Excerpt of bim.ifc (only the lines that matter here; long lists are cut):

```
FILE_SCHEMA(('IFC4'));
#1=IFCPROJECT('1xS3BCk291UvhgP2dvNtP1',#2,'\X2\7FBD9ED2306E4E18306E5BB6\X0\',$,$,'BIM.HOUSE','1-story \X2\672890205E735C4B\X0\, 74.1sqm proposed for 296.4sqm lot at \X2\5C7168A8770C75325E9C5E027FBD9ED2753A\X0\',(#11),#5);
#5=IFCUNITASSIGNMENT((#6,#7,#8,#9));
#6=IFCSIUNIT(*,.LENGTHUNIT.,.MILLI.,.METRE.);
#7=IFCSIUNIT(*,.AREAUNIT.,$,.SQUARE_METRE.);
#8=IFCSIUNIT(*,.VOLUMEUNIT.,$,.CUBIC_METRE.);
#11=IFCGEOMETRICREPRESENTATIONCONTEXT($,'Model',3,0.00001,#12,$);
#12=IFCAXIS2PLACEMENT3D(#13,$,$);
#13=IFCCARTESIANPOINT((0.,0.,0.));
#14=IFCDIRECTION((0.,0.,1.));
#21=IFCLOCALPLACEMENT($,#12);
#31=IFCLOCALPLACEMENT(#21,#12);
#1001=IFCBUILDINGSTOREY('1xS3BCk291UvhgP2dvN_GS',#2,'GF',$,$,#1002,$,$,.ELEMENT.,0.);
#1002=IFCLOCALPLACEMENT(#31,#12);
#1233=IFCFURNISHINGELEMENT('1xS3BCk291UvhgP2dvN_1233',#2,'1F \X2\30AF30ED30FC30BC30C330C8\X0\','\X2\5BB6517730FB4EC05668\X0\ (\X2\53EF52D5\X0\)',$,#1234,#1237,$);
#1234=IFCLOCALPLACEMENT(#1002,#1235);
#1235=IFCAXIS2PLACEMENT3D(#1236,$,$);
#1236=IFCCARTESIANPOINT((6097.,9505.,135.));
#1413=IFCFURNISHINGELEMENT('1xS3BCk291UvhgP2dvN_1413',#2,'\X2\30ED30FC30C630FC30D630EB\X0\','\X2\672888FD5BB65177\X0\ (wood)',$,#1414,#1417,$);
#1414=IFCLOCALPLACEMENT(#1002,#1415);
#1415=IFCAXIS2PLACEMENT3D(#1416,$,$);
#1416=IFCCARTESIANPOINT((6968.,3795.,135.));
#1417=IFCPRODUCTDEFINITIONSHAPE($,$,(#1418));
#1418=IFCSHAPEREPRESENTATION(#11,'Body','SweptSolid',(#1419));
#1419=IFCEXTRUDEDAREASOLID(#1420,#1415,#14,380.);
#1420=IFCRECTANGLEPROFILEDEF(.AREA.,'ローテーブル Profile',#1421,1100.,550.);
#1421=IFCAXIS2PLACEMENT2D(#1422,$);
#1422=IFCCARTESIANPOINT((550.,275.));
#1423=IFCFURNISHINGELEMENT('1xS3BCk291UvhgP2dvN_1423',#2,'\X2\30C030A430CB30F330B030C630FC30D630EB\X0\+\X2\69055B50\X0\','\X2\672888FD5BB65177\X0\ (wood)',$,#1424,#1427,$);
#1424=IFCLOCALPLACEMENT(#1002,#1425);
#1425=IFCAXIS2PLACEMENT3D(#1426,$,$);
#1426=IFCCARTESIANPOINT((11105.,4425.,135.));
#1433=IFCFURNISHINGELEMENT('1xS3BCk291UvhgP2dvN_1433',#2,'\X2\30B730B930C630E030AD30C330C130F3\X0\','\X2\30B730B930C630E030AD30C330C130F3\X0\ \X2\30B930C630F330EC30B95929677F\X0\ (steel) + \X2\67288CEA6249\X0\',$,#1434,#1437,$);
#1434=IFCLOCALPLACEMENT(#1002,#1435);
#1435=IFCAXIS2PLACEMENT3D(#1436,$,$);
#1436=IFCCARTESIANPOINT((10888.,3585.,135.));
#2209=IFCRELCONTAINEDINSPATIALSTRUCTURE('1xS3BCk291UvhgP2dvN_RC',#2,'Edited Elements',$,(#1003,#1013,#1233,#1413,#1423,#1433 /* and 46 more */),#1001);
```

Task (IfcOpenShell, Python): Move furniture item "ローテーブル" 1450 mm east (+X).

```python
import ifcopenshell
import ifcopenshell.api.geometry
import ifcopenshell.util.placement
import ifcopenshell.util.unit

model = ifcopenshell.open("bim.ifc")
unit_scale = ifcopenshell.util.unit.calculate_unit_scale(model)

item = model.by_guid("1xS3BCk291UvhgP2dvN_1413")
matrix = ifcopenshell.util.placement.get_local_placement(item.ObjectPlacement)
matrix[0, 3] += 1.45 / unit_scale
ifcopenshell.api.geometry.edit_object_placement(model, product=item, matrix=matrix, is_si=False)

print(ifcopenshell.util.placement.get_local_placement(item.ObjectPlacement).round(3) + 0.0)

model.write("bim_v2.ifc")
```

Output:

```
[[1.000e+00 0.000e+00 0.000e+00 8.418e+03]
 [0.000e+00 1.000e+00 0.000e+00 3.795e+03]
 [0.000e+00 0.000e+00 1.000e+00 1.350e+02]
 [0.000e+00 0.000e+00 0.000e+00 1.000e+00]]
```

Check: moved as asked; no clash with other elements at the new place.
